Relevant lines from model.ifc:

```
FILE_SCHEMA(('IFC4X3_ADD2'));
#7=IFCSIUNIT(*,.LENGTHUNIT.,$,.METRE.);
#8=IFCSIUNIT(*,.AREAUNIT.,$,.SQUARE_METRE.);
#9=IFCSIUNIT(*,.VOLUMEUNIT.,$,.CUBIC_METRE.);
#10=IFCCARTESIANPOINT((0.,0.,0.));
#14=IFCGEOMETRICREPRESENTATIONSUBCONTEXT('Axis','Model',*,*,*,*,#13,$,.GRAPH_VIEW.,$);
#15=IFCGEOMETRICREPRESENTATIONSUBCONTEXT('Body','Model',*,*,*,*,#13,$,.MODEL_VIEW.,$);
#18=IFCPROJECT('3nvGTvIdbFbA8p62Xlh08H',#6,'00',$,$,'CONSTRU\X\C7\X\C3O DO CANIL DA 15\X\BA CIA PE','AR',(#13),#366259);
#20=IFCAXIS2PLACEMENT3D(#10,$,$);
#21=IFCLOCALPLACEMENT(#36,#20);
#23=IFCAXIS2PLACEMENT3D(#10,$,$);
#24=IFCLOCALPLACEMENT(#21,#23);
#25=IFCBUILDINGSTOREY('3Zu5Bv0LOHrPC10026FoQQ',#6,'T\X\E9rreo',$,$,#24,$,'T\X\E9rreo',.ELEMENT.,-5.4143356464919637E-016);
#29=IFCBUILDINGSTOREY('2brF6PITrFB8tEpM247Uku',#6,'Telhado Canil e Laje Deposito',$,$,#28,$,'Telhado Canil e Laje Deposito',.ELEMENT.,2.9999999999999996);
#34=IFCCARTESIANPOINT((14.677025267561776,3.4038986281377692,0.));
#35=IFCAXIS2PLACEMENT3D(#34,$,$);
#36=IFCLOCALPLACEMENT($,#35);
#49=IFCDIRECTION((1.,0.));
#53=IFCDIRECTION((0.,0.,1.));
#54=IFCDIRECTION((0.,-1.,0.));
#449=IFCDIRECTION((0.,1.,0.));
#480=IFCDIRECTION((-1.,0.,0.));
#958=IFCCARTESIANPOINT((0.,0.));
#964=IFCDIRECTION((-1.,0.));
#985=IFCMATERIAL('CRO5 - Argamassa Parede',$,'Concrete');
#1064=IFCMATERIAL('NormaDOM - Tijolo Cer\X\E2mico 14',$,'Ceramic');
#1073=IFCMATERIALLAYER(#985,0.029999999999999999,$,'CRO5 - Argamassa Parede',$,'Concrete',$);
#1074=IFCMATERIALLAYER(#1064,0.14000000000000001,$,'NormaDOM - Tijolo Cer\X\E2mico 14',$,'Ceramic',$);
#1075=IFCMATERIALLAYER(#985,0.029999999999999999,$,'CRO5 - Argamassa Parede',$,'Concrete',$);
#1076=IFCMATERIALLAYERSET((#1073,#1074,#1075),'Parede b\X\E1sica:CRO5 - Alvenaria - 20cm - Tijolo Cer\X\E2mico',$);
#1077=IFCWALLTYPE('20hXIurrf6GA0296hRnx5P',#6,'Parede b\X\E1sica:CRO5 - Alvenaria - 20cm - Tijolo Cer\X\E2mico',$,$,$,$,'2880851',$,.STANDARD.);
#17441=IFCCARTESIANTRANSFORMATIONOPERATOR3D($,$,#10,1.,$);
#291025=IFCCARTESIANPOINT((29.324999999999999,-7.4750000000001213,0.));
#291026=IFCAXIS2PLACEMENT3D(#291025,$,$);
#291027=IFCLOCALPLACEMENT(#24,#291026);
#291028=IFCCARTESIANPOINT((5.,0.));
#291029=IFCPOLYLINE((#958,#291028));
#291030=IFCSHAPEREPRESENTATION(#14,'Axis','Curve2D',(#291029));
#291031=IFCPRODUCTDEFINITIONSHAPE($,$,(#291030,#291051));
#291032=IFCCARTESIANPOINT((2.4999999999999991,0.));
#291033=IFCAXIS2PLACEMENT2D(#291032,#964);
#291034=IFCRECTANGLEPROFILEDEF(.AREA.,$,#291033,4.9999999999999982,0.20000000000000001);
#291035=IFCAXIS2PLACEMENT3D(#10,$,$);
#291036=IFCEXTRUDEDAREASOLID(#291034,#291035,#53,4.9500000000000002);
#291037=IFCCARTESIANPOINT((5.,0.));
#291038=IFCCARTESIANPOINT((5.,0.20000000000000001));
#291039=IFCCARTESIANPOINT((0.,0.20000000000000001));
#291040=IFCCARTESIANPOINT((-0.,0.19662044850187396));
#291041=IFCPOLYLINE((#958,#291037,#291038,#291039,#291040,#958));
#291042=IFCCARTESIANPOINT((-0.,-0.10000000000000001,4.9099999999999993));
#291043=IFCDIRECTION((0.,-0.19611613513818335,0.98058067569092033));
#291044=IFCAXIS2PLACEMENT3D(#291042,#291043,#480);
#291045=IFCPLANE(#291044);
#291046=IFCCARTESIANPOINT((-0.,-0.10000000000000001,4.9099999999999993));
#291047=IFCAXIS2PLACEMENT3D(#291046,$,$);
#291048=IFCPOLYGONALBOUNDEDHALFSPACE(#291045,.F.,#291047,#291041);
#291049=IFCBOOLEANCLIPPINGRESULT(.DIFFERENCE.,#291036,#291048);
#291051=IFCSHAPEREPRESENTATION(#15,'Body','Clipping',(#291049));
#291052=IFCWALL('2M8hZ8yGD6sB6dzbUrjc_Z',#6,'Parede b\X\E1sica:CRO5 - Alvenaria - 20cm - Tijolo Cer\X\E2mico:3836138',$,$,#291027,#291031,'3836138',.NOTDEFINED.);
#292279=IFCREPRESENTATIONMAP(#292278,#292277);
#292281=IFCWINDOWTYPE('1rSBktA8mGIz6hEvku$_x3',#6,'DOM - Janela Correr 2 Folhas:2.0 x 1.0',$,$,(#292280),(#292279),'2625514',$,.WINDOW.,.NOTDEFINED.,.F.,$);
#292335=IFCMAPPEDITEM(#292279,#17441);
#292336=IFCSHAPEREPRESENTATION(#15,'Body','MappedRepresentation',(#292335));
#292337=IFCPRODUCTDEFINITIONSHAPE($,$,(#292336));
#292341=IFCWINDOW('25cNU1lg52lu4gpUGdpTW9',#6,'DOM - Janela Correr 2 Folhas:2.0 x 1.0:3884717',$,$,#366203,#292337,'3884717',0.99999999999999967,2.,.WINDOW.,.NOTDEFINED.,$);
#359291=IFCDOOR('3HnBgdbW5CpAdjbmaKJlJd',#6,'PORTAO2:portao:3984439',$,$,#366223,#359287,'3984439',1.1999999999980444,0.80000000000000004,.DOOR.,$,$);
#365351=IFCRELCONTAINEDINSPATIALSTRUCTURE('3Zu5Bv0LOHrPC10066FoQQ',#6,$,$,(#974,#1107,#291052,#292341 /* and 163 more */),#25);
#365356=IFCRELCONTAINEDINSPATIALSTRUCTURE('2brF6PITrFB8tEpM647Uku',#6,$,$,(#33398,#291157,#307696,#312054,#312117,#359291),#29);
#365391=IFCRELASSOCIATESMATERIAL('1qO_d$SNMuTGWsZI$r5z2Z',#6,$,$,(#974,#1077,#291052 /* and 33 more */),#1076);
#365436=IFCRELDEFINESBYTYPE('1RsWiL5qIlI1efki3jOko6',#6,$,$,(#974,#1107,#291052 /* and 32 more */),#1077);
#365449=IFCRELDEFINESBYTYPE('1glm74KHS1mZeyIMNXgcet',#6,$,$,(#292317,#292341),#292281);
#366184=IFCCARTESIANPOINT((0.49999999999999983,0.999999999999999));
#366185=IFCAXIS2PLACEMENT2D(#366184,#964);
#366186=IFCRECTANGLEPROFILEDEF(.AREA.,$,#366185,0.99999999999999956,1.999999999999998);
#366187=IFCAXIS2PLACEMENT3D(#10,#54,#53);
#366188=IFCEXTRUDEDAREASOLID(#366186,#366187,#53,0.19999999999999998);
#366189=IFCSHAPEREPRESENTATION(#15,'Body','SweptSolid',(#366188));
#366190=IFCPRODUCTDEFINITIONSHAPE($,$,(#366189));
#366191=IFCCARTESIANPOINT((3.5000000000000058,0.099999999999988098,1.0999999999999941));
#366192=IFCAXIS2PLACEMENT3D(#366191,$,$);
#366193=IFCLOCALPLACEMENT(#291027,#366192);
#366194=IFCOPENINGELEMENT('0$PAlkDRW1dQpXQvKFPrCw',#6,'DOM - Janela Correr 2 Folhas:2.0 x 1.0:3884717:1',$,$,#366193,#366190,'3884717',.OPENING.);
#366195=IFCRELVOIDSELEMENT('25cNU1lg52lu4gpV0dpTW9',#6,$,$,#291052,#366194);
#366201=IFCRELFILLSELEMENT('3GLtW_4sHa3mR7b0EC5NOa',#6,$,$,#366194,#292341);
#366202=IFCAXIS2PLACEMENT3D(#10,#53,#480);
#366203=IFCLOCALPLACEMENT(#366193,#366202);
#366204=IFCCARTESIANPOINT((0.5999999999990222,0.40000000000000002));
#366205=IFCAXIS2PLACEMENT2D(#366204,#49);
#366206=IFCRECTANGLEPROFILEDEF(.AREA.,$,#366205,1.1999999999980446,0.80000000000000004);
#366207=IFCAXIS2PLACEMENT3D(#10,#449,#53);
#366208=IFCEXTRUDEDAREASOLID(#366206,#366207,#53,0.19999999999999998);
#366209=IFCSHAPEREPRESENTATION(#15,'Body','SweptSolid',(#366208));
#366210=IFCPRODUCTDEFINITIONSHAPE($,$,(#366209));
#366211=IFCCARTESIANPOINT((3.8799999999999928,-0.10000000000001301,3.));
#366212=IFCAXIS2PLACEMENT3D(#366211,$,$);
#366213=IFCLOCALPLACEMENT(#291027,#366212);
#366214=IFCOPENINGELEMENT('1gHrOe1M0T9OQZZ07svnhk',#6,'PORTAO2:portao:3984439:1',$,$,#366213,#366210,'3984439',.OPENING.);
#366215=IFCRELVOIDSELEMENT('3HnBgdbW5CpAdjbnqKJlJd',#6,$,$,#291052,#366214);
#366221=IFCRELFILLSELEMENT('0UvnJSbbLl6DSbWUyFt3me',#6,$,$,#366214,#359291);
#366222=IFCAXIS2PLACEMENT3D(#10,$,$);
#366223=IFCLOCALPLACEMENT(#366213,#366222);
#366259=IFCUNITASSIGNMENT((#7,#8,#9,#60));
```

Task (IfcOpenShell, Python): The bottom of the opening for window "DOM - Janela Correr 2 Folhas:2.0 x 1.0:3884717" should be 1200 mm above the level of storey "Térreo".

```python
import numpy as np
import ifcopenshell
import ifcopenshell.api.geometry
import ifcopenshell.geom
import ifcopenshell.util.element
import ifcopenshell.util.placement
import ifcopenshell.util.shape
import ifcopenshell.util.unit

model = ifcopenshell.open("model.ifc")
unit_scale = ifcopenshell.util.unit.calculate_unit_scale(model)

window = model.by_id(292341)
opening = window.FillsVoids[0].RelatingOpeningElement
storey = ifcopenshell.util.element.get_container(window, ifc_class="IfcBuildingStorey")
level = ifcopenshell.util.placement.get_local_placement(storey.ObjectPlacement)[2, 3]

# The opening's origin need not be at the sill, so measure its lowest point.
shape = ifcopenshell.geom.create_shape(ifcopenshell.geom.settings(), opening)
bottom = ifcopenshell.util.shape.get_shape_bottom_elevation(shape, shape.geometry) / unit_scale
dz = level + 1.2 / unit_scale - bottom

shift = np.array([0.0, 0.0, dz])
# The window is placed relative to its opening, so it follows when the opening moves.
matrix = ifcopenshell.util.placement.get_local_placement(opening.ObjectPlacement)
matrix[:3, 3] += shift
ifcopenshell.api.geometry.edit_object_placement(
    model, product=opening, matrix=matrix, is_si=False, should_transform_children=True
)

print(f"moved by {dz * unit_scale:+.3f} m")

model.write("model-out.ifc")
```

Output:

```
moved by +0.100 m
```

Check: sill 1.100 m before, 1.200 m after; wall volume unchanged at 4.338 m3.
